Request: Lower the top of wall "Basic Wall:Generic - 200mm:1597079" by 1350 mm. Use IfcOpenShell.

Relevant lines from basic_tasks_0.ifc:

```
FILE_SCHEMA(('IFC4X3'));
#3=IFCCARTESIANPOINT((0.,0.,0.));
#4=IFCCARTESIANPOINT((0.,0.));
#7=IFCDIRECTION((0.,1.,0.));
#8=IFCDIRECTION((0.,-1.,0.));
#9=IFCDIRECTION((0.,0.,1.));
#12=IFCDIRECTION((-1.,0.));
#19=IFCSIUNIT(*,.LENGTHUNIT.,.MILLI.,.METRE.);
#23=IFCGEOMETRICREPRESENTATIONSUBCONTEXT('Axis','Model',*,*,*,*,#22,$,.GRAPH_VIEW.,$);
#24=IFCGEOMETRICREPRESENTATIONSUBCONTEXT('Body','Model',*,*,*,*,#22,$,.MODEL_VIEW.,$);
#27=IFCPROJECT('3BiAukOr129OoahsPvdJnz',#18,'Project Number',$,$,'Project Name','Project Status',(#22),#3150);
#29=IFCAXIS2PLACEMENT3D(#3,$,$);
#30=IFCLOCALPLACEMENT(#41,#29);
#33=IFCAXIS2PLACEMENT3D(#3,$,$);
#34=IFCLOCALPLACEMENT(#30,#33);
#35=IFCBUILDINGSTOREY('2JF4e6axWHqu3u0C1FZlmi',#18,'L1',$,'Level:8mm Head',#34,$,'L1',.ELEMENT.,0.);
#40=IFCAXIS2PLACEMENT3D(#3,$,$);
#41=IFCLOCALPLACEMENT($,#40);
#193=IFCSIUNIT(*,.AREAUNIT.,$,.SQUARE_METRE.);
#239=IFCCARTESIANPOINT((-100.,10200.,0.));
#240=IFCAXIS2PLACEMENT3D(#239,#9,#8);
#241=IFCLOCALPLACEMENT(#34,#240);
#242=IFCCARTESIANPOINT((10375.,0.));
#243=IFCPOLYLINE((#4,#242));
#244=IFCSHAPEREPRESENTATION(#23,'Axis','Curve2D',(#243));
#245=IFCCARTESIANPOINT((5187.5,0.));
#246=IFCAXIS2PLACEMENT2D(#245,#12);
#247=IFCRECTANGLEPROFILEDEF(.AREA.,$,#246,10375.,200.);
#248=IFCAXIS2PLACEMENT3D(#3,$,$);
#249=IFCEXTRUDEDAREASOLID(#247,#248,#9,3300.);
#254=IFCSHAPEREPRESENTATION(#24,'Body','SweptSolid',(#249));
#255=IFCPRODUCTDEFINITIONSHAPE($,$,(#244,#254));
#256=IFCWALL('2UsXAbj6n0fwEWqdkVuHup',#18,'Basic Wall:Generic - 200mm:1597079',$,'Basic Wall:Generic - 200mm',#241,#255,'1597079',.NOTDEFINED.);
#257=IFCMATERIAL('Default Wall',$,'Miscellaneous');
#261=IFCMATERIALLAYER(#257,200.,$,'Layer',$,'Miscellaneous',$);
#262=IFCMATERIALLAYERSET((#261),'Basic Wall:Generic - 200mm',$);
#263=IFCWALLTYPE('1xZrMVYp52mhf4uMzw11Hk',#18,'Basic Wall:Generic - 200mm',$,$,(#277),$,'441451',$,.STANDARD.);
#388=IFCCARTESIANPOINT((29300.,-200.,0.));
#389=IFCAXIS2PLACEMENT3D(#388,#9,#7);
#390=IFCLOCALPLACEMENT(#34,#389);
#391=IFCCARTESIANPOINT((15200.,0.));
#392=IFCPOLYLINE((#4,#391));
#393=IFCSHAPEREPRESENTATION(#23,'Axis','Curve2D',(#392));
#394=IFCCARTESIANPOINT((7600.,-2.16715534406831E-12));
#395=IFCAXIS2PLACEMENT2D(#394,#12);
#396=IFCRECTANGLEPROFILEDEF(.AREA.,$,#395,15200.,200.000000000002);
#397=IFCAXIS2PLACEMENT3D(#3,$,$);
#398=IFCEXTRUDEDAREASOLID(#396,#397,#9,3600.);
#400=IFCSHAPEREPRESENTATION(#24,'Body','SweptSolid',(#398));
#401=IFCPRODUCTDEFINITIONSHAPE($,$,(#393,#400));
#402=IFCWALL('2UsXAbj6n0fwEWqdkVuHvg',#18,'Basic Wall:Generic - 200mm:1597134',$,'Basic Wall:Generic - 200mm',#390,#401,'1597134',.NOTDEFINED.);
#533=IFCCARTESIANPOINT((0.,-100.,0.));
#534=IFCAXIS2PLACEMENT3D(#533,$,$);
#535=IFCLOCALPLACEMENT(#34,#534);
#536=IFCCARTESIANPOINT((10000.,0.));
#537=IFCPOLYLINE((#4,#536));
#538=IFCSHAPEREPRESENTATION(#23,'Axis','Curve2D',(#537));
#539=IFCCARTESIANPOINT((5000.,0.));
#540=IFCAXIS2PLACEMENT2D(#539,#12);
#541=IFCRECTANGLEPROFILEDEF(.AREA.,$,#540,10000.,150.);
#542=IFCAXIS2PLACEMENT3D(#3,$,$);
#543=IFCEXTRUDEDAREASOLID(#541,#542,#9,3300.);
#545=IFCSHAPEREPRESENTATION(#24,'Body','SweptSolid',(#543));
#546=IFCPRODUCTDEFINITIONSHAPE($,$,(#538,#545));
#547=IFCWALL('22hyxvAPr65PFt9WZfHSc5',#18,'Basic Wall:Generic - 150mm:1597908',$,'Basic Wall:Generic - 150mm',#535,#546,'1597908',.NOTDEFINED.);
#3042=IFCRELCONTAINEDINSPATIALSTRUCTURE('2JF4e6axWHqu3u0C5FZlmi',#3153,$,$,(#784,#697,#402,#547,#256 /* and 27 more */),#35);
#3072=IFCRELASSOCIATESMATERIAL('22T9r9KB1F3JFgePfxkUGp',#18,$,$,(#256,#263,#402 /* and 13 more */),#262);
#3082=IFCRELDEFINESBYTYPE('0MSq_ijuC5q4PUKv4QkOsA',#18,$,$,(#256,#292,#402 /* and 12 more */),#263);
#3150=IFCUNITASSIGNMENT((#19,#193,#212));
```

```python
import ifcopenshell
import ifcopenshell.geom
import ifcopenshell.util.representation
import ifcopenshell.util.shape

model = ifcopenshell.open("basic_tasks_0.ifc")
settings = ifcopenshell.geom.settings()


def volume(element):
    """Net volume in cubic metres, openings subtracted."""
    shape = ifcopenshell.geom.create_shape(settings, element)
    return ifcopenshell.util.shape.get_volume(shape.geometry)


wall = model.by_guid("2UsXAbj6n0fwEWqdkVuHup")
before = volume(wall)

body = ifcopenshell.util.representation.get_representation(wall, "Model", "Body")
solid = body.Items[0]
old_height = solid.Depth
solid.Depth -= 1350.0
after = volume(wall)

print(f"height {old_height:g} -> {solid.Depth:g}, volume {before:.3f} -> {after:.3f} m3")

model.write("basic_tasks_0_v2.ifc")
```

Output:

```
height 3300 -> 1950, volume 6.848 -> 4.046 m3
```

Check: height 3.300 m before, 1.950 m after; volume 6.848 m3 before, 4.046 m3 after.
